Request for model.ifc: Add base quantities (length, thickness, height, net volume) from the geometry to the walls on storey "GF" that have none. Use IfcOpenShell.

First a look at what the model holds.

```python
import ifcopenshell
import ifcopenshell.util.element
import ifcopenshell.util.unit

model = ifcopenshell.open("model.ifc")
print(model.schema)
for unit_type in ("LENGTHUNIT", "AREAUNIT", "VOLUMEUNIT"):
    print(unit_type, ifcopenshell.util.unit.calculate_unit_scale(model, unit_type))
storey = next(s for s in model.by_type("IfcBuildingStorey") if s.Name == "GF")
walls = [e for e in ifcopenshell.util.element.get_decomposition(storey) if e.is_a("IfcWall")]
for e in sorted(walls, key=lambda e: e.id()):
    print(e.id(), e.is_a(), e.Name, list(ifcopenshell.util.element.get_psets(e, qtos_only=True)), sep=" | ")
```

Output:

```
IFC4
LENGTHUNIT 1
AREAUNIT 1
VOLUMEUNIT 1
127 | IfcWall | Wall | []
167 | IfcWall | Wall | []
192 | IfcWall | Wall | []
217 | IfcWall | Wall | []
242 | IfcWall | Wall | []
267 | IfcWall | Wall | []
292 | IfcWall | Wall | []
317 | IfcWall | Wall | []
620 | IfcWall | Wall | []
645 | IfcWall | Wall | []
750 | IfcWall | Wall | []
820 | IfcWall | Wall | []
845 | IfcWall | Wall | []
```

```python
import ifcopenshell
import ifcopenshell.api.pset
import ifcopenshell.geom
import ifcopenshell.util.element
import ifcopenshell.util.shape
import ifcopenshell.util.unit

model = ifcopenshell.open("model.ifc")
unit_scale = ifcopenshell.util.unit.calculate_unit_scale(model)
volume_scale = ifcopenshell.util.unit.calculate_unit_scale(model, "VOLUMEUNIT")
settings = ifcopenshell.geom.settings()

storey = next(s for s in model.by_type("IfcBuildingStorey") if s.Name == "GF")
walls = [e for e in ifcopenshell.util.element.get_decomposition(storey) if e.is_a("IfcWall")]

for e in sorted(walls, key=lambda e: e.id()):
    if ifcopenshell.util.element.get_psets(e, qtos_only=True, should_inherit=False):
        continue
    # Geometry comes back in metres, in the element's own axes.
    shape = ifcopenshell.geom.create_shape(settings, e)
    values = {
        "Length": ifcopenshell.util.shape.get_x(shape.geometry) / unit_scale,
        "Width": ifcopenshell.util.shape.get_y(shape.geometry) / unit_scale,
        "Height": ifcopenshell.util.shape.get_z(shape.geometry) / unit_scale,
        "NetVolume": ifcopenshell.util.shape.get_volume(shape.geometry) / volume_scale,
    }
    qto = ifcopenshell.api.pset.add_qto(model, product=e, name="Qto_WallBaseQuantities")
    ifcopenshell.api.pset.edit_qto(model, qto=qto, properties=values)
    print(e.id(), {k: round(v, 3) for k, v in values.items()})

model.write("model_updated.ifc")
```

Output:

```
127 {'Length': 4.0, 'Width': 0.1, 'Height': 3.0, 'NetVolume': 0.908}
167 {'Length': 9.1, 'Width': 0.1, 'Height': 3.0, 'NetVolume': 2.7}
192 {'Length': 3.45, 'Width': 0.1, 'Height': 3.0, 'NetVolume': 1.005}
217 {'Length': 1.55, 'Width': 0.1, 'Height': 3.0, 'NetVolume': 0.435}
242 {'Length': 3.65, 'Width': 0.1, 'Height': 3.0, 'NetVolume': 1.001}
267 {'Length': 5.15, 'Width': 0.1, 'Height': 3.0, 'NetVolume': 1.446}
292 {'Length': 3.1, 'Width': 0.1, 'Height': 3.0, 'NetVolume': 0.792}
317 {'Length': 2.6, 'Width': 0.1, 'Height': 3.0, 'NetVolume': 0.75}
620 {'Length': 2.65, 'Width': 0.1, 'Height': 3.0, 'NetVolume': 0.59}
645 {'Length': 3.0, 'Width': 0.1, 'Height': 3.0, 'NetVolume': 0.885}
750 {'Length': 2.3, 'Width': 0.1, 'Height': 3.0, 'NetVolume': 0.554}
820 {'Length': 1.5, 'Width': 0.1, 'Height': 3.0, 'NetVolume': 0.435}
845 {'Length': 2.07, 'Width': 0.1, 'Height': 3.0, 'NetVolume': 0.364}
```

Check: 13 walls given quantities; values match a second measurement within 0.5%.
